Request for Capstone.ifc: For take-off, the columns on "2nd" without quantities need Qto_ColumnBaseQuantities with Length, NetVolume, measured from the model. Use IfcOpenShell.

First a look at what the model holds.

```python
import ifcopenshell
import ifcopenshell.util.element
import ifcopenshell.util.unit

model = ifcopenshell.open("Capstone.ifc")
print(model.schema)
for unit_type in ("LENGTHUNIT", "AREAUNIT", "VOLUMEUNIT"):
    print(unit_type, ifcopenshell.util.unit.calculate_unit_scale(model, unit_type))
storey = next(s for s in model.by_type("IfcBuildingStorey") if s.Name == "2nd")
columns = [e for e in ifcopenshell.util.element.get_decomposition(storey) if e.is_a("IfcColumn")]
for e in sorted(columns, key=lambda e: e.id()):
    print(e.id(), e.is_a(), e.Name, list(ifcopenshell.util.element.get_psets(e, qtos_only=True)), sep=" | ")
```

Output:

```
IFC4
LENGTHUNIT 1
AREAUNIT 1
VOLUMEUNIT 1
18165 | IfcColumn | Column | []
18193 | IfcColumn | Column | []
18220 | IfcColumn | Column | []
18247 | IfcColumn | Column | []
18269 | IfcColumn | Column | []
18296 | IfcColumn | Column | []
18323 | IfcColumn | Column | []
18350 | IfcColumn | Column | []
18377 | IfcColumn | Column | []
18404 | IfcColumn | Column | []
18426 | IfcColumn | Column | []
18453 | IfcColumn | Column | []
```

```python
import ifcopenshell
import ifcopenshell.api.pset
import ifcopenshell.geom
import ifcopenshell.util.element
import ifcopenshell.util.shape
import ifcopenshell.util.unit

model = ifcopenshell.open("Capstone.ifc")
unit_scale = ifcopenshell.util.unit.calculate_unit_scale(model)
volume_scale = ifcopenshell.util.unit.calculate_unit_scale(model, "VOLUMEUNIT")
settings = ifcopenshell.geom.settings()

storey = next(s for s in model.by_type("IfcBuildingStorey") if s.Name == "2nd")
columns = [e for e in ifcopenshell.util.element.get_decomposition(storey) if e.is_a("IfcColumn")]

for e in sorted(columns, key=lambda e: e.id()):
    if ifcopenshell.util.element.get_psets(e, qtos_only=True, should_inherit=False):
        continue
    # Geometry comes back in metres, in the element's own axes.
    shape = ifcopenshell.geom.create_shape(settings, e)
    values = {
        "Length": ifcopenshell.util.shape.get_z(shape.geometry) / unit_scale,
        "NetVolume": ifcopenshell.util.shape.get_volume(shape.geometry) / volume_scale,
    }
    qto = ifcopenshell.api.pset.add_qto(model, product=e, name="Qto_ColumnBaseQuantities")
    ifcopenshell.api.pset.edit_qto(model, qto=qto, properties=values)
    print(e.id(), {k: round(v, 3) for k, v in values.items()})

model.write("Capstone-out.ifc")
```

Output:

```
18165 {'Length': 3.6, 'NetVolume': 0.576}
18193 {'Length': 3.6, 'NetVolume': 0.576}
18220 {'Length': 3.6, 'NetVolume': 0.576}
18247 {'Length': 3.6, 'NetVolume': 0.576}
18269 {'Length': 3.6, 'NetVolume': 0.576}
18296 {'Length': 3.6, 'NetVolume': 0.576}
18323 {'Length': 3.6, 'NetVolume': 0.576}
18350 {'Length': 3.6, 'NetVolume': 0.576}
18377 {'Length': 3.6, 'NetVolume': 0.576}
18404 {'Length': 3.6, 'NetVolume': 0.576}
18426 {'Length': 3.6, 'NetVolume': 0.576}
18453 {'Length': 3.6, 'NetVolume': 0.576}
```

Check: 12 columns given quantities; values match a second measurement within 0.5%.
